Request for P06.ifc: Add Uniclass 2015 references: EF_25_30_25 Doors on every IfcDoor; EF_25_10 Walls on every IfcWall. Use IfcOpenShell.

First a look at what the model holds.

```python
import ifcopenshell

model = ifcopenshell.open("P06.ifc")
print(model.schema)
print("classifications:", [c.Name for c in model.by_type("IfcClassification")])
for ifc_class in ("IfcDoor", "IfcRoof", "IfcStair", "IfcWall", "IfcWindow"):
    print(ifc_class, len(model.by_type(ifc_class)))
```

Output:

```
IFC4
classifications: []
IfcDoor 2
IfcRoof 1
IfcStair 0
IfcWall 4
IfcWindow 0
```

```python
import ifcopenshell
import ifcopenshell.api.classification

model = ifcopenshell.open("P06.ifc")

system = ifcopenshell.api.classification.add_classification(model, classification="Uniclass 2015")

codes = {
    "IfcDoor": ("EF_25_30_25", "Doors"),
    "IfcWall": ("EF_25_10", "Walls"),
}
for ifc_class, (code, name) in codes.items():
    products = model.by_type(ifc_class)
    ifcopenshell.api.classification.add_reference(
        model, products=products, classification=system, identification=code, name=name
    )
    print(code, len(products))

model.write("P06_v2.ifc")
```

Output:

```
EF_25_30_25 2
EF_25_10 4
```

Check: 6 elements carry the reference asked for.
